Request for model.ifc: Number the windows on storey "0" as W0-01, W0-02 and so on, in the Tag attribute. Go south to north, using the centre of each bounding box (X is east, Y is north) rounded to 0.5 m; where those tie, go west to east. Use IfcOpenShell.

First a look at what the model holds.

```python
import ifcopenshell
import ifcopenshell.util.element
import ifcopenshell.util.placement

model = ifcopenshell.open("model.ifc")
print(model.schema)
storey = next(s for s in model.by_type("IfcBuildingStorey") if s.Name == "0")
windows = [e for e in ifcopenshell.util.element.get_decomposition(storey) if e.is_a("IfcWindow")]
for e in sorted(windows, key=lambda e: e.id()):
    origin = ifcopenshell.util.placement.get_local_placement(e.ObjectPlacement)[:3, 3]
    print(e.id(), e.Tag, e.Name, origin.round(2) + 0.0, sep=" | ")
```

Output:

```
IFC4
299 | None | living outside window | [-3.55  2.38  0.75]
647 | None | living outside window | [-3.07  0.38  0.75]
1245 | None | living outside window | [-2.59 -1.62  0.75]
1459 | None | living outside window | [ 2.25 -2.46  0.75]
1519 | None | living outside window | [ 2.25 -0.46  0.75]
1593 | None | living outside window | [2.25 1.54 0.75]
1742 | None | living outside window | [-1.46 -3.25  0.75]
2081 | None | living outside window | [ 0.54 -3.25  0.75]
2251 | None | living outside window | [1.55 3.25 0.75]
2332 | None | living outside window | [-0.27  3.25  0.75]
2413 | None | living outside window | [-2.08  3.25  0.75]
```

```python
import ifcopenshell
import ifcopenshell.geom
import ifcopenshell.util.element
import ifcopenshell.util.shape

model = ifcopenshell.open("model.ifc")
settings = ifcopenshell.geom.settings()
settings.set("use-world-coords", True)


def centre(element):
    shape = ifcopenshell.geom.create_shape(settings, element)
    return ifcopenshell.util.shape.get_bbox_centroid(shape.geometry)


storey = next(s for s in model.by_type("IfcBuildingStorey") if s.Name == "0")
windows = [e for e in ifcopenshell.util.element.get_decomposition(storey) if e.is_a("IfcWindow")]

# Insertion points can sit at a corner or the storey origin, so sort by the geometry (in metres).
centres = {e: centre(e) for e in windows}
windows.sort(key=lambda e: (round(centres[e][1] / 0.5), centres[e][0]))

for i, e in enumerate(windows, start=1):
    number = f"W0-{i:02d}"
    e.Tag = number
    print(e.id(), number)

model.write("model_edited.ifc")
```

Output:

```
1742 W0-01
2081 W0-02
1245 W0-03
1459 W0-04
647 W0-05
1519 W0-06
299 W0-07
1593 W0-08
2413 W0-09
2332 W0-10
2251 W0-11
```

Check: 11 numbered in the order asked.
